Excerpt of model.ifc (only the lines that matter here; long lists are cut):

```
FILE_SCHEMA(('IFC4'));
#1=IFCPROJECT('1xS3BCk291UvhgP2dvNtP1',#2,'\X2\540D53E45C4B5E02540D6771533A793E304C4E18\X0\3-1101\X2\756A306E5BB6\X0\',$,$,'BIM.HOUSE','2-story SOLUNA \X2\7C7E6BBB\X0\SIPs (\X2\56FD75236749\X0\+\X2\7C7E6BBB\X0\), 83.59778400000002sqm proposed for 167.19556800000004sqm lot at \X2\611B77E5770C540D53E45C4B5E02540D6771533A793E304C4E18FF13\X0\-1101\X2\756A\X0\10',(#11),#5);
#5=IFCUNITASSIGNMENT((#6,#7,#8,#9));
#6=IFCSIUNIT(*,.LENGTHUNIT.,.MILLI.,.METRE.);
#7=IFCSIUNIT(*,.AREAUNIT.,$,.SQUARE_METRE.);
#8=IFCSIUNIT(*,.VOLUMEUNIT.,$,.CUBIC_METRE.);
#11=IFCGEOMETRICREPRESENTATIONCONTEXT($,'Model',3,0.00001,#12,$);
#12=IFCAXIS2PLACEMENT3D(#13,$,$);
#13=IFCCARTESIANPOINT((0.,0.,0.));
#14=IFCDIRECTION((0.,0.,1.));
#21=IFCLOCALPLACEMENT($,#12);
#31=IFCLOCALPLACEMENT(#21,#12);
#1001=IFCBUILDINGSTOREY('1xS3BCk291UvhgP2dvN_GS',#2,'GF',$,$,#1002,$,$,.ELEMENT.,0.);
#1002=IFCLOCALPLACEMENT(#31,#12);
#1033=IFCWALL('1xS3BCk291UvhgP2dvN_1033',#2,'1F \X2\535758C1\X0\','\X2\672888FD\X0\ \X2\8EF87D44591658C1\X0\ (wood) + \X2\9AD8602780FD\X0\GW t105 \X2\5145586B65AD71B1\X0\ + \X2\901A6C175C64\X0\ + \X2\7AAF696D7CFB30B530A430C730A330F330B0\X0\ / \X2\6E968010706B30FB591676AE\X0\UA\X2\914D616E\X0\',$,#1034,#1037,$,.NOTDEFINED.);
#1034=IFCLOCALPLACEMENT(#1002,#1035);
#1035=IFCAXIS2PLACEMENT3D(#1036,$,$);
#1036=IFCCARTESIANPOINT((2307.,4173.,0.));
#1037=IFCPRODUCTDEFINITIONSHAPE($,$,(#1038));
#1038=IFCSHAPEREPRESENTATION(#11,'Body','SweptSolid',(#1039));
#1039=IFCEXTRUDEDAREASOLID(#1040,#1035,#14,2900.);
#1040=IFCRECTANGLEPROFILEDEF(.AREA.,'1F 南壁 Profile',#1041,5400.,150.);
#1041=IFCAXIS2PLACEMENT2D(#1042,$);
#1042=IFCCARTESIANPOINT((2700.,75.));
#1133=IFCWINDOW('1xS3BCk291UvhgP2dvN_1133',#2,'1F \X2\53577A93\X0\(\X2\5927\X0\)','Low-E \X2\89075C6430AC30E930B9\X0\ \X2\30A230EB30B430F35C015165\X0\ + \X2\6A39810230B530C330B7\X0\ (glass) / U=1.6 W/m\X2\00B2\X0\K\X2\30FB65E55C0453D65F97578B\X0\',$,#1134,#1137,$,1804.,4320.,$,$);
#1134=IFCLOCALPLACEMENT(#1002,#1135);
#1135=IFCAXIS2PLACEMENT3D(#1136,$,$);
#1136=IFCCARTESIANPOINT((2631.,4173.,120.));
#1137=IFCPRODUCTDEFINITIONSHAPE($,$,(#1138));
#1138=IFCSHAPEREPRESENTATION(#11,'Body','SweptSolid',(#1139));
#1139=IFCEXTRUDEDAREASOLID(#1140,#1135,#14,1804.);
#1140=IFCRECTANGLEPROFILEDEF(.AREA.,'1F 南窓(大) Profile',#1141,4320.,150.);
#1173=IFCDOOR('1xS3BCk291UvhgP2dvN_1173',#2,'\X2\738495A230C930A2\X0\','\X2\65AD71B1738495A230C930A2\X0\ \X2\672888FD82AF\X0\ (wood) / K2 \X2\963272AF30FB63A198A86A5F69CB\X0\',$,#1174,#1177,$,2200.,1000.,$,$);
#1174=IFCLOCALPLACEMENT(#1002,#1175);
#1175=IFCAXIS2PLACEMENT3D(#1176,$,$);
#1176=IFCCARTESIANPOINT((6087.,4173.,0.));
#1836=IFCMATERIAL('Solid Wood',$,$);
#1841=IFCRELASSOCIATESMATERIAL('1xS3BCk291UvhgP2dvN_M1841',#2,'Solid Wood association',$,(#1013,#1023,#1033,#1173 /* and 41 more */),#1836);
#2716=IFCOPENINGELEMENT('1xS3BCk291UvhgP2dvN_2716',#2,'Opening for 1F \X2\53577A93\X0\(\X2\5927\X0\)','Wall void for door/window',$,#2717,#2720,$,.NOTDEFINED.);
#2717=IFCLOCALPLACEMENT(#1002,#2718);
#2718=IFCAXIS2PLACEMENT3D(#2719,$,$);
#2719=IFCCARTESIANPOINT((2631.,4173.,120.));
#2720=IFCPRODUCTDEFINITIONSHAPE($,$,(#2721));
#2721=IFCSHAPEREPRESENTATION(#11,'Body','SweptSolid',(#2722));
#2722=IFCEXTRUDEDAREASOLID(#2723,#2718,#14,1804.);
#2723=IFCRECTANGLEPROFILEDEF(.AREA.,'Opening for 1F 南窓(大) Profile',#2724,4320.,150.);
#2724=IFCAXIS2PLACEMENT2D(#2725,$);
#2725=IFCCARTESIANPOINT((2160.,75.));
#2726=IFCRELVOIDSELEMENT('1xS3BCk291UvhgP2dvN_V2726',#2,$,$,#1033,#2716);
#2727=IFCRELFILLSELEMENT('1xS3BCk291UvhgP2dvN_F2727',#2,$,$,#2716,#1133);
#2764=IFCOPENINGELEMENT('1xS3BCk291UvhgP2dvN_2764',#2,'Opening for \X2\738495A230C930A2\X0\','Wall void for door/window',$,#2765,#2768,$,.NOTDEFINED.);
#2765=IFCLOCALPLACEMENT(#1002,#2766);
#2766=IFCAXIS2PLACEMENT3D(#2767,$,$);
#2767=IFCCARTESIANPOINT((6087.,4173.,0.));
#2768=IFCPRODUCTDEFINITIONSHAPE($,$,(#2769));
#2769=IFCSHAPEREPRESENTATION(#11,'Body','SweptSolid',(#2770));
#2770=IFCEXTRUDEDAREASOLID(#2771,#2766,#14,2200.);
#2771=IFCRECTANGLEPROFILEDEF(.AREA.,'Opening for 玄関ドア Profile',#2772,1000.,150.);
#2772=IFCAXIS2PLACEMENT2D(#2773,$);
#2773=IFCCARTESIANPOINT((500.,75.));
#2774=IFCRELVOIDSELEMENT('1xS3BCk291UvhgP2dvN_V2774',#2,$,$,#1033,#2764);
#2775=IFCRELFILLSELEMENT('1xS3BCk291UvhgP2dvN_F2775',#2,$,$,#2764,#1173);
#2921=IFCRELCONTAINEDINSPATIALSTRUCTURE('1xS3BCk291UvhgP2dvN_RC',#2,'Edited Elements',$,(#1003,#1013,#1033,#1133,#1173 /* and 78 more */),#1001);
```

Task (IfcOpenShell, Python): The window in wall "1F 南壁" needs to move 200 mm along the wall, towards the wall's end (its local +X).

```python
import ifcopenshell
import ifcopenshell.api.geometry
import ifcopenshell.util.placement

model = ifcopenshell.open("model.ifc")

window = model.by_guid("1xS3BCk291UvhgP2dvN_1133")
opening = window.FillsVoids[0].RelatingOpeningElement
wall = opening.VoidsElements[0].RelatingBuildingElement

wall_matrix = ifcopenshell.util.placement.get_local_placement(wall.ObjectPlacement)
shift = wall_matrix[:3, 0] * 200.0
before = ifcopenshell.util.placement.get_local_placement(window.ObjectPlacement)[:3, 3].copy()

# The window is not placed relative to its opening, so move both.
for product in (opening, window):
    matrix = ifcopenshell.util.placement.get_local_placement(product.ObjectPlacement)
    matrix[:3, 3] += shift
    ifcopenshell.api.geometry.edit_object_placement(model, product=product, matrix=matrix, is_si=False)

after = ifcopenshell.util.placement.get_local_placement(window.ObjectPlacement)[:3, 3]
print("window moved by", (after - before).round(3) + 0.0)

model.write("model_v2.ifc")
```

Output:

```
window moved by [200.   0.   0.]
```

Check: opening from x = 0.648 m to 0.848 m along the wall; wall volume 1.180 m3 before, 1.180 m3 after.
